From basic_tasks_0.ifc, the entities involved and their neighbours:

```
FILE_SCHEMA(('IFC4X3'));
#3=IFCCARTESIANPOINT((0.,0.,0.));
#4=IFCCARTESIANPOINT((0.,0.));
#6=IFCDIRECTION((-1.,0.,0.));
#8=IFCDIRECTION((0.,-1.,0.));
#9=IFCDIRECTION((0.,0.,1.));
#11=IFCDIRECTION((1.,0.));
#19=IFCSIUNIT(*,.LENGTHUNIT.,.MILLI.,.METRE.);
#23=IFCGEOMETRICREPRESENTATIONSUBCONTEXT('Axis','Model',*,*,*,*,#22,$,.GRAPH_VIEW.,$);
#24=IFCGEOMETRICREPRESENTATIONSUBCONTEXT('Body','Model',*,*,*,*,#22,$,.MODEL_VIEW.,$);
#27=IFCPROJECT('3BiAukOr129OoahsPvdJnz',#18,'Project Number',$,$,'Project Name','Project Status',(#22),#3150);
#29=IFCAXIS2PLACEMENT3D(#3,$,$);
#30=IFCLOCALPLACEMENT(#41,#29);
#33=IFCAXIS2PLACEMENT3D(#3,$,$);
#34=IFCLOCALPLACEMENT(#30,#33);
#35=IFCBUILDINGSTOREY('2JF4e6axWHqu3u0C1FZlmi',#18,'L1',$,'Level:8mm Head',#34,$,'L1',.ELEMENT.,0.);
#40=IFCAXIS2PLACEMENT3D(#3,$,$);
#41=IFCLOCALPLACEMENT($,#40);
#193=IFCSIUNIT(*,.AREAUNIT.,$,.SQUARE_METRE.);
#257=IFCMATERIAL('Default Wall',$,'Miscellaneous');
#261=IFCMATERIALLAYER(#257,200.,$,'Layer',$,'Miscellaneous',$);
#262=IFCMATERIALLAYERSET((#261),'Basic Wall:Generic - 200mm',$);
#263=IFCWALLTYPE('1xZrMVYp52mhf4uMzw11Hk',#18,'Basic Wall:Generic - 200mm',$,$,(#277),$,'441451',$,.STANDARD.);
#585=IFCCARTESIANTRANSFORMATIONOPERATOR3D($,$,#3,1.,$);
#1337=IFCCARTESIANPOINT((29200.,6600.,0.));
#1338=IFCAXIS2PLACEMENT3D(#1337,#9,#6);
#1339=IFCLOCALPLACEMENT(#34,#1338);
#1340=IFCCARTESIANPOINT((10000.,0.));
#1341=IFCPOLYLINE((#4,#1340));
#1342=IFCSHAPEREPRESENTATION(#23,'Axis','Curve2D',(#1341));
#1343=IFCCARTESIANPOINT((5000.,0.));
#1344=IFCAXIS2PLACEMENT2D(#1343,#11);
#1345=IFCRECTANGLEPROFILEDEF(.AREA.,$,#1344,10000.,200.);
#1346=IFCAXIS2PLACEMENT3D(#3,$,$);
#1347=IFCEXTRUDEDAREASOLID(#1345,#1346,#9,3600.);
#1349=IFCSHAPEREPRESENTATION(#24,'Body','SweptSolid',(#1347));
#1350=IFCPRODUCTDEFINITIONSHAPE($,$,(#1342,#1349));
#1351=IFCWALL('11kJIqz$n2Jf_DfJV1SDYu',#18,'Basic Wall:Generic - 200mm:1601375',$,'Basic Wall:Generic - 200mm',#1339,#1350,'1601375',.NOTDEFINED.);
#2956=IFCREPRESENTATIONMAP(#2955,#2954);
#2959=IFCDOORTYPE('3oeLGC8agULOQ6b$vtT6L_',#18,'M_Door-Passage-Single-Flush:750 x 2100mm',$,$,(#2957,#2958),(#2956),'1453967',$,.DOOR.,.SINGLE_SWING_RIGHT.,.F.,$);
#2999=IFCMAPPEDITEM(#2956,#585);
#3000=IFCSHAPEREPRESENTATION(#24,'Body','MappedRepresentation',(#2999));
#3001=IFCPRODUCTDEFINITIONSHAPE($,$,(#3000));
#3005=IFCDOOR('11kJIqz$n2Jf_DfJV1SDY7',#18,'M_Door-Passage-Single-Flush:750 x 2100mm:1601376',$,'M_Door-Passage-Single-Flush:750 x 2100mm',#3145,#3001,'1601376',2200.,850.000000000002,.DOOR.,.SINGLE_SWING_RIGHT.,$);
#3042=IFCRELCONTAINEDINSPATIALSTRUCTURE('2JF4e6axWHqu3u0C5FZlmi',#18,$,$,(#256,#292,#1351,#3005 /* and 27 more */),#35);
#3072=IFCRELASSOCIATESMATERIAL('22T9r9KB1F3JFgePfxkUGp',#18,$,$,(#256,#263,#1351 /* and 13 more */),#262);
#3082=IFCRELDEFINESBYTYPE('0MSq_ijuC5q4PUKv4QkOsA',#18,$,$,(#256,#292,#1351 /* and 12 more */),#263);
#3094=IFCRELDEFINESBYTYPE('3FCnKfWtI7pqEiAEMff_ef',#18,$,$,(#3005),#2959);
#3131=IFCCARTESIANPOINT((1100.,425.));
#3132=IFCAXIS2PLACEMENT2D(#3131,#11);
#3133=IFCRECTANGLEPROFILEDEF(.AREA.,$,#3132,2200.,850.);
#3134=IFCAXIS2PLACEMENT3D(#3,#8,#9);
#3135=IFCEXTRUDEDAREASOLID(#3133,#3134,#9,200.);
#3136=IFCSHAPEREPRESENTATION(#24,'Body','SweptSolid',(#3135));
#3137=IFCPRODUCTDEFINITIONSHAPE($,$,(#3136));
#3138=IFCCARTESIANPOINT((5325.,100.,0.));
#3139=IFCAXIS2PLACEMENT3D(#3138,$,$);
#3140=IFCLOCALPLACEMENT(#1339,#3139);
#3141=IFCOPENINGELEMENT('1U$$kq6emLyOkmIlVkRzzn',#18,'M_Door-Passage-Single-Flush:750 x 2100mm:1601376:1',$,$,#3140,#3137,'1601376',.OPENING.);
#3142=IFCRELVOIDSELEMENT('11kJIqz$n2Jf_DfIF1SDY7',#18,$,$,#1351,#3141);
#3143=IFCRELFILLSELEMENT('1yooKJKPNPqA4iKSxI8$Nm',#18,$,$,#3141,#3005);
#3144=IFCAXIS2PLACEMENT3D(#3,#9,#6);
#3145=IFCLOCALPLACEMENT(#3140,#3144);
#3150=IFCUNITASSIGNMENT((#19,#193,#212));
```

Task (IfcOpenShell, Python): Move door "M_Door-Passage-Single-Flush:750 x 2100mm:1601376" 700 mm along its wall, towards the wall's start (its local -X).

```python
import ifcopenshell
import ifcopenshell.api.geometry
import ifcopenshell.util.placement
import ifcopenshell.util.unit

model = ifcopenshell.open("basic_tasks_0.ifc")
unit_scale = ifcopenshell.util.unit.calculate_unit_scale(model)

door = model.by_guid("11kJIqz$n2Jf_DfJV1SDY7")
opening = door.FillsVoids[0].RelatingOpeningElement
wall = opening.VoidsElements[0].RelatingBuildingElement

wall_matrix = ifcopenshell.util.placement.get_local_placement(wall.ObjectPlacement)
shift = wall_matrix[:3, 0] * -0.7 / unit_scale
before = ifcopenshell.util.placement.get_local_placement(door.ObjectPlacement)[:3, 3].copy()

# The door is placed relative to its opening, so it follows when the opening moves.
matrix = ifcopenshell.util.placement.get_local_placement(opening.ObjectPlacement)
matrix[:3, 3] += shift
ifcopenshell.api.geometry.edit_object_placement(
    model, product=opening, matrix=matrix, is_si=False, should_transform_children=True
)

after = ifcopenshell.util.placement.get_local_placement(door.ObjectPlacement)[:3, 3]
print("door moved by", (after - before).round(3) + 0.0)

model.write("basic_tasks_0_edited.ifc")
```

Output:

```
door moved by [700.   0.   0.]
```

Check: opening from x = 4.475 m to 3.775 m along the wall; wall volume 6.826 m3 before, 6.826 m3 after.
